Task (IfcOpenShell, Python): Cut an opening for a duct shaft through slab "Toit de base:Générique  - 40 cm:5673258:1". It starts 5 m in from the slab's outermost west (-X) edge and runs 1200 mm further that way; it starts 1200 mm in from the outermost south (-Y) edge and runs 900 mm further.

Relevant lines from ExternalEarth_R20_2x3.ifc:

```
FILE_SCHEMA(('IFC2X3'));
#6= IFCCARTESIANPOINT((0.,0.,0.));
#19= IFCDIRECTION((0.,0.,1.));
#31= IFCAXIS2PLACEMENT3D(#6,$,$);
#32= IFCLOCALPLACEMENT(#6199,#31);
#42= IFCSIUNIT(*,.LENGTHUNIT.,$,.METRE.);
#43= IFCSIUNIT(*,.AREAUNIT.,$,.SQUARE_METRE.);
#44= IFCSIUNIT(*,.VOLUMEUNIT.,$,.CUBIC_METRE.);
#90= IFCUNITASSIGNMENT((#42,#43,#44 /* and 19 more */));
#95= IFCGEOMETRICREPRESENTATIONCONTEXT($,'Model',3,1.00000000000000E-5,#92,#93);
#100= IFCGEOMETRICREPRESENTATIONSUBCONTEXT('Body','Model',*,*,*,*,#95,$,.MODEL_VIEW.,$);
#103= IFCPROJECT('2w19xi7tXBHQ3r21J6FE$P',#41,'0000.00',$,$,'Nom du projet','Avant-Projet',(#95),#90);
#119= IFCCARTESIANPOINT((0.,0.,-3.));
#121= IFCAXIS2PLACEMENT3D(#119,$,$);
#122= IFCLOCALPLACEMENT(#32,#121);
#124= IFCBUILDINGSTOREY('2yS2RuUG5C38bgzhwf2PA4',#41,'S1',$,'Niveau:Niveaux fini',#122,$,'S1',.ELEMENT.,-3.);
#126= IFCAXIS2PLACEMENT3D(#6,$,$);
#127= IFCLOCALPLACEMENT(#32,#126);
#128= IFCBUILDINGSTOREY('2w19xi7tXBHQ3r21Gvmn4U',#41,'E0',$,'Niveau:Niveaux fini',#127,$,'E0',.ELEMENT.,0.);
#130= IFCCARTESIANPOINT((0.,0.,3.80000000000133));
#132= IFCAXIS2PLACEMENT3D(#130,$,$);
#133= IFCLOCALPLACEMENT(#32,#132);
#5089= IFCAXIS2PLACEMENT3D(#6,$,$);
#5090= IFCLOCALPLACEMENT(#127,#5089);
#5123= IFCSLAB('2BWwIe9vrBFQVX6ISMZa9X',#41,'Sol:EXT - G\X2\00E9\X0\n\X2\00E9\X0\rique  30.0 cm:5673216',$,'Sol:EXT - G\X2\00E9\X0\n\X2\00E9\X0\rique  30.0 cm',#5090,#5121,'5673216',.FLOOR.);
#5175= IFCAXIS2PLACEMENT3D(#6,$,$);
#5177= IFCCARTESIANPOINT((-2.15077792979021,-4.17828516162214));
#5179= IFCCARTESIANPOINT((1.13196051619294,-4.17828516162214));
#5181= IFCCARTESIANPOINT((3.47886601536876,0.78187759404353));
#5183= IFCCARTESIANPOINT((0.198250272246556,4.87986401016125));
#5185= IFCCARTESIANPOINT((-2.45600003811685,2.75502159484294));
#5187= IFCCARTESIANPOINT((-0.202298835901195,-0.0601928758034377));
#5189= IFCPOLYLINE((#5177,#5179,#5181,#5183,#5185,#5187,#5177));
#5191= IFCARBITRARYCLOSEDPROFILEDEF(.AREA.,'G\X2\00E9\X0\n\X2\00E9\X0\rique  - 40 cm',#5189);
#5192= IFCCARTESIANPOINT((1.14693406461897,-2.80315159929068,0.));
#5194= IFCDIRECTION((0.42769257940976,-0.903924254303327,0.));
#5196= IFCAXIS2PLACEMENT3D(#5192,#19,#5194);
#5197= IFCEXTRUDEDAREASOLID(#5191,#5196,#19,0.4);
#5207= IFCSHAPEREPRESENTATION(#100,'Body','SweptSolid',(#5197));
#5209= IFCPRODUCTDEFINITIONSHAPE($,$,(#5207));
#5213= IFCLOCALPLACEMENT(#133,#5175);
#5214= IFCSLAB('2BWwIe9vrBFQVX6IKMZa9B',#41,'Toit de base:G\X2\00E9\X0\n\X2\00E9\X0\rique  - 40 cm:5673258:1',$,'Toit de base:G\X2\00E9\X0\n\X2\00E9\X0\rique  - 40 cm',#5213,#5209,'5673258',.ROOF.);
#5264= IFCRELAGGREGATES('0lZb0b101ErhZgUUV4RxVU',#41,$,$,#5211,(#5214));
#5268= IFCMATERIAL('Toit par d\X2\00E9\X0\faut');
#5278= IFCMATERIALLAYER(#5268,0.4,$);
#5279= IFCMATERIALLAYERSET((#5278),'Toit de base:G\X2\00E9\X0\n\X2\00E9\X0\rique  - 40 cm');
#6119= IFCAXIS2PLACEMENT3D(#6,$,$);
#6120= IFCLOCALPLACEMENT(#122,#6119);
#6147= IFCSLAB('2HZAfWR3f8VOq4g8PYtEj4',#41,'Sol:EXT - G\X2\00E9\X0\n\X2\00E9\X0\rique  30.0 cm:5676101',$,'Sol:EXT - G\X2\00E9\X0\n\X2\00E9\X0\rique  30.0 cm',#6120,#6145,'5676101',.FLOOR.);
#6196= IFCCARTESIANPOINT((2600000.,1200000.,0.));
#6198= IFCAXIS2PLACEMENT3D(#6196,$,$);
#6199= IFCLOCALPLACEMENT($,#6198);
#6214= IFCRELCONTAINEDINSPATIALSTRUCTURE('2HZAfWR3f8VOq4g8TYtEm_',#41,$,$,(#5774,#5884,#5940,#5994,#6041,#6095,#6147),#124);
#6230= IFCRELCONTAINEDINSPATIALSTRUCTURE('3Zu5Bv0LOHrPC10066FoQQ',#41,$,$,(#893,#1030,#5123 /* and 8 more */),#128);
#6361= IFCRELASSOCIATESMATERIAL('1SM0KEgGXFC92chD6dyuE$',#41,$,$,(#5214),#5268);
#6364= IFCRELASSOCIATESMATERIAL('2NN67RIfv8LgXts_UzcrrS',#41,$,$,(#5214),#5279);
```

```python
import numpy as np
import ifcopenshell
import ifcopenshell.api.feature
import ifcopenshell.api.geometry
import ifcopenshell.api.root
import ifcopenshell.geom
import ifcopenshell.util.placement
import ifcopenshell.util.representation
import ifcopenshell.util.shape
import ifcopenshell.util.unit

model = ifcopenshell.open("ExternalEarth_R20_2x3.ifc")
unit_scale = ifcopenshell.util.unit.calculate_unit_scale(model)
settings = ifcopenshell.geom.settings()


def volume(element):
    """Net volume in cubic metres, openings subtracted."""
    shape = ifcopenshell.geom.create_shape(settings, element)
    return ifcopenshell.util.shape.get_volume(shape.geometry)


slab = model.by_guid("2BWwIe9vrBFQVX6IKMZa9B")
before = volume(slab)

# Extent in the slab's own axes, in metres. The edges named are its -X and -Y sides.
slab_shape = ifcopenshell.geom.create_shape(settings, slab)
vertices = ifcopenshell.util.shape.get_vertices(slab_shape.geometry)
x_min, y_min, bottom = vertices.min(axis=0)
top = vertices[:, 2].max()

opening = ifcopenshell.api.root.create_entity(model, ifc_class="IfcOpeningElement", name="Duct shaft opening")
context = ifcopenshell.util.representation.get_context(model, "Model", "Body", "MODEL_VIEW")
width, depth = 1.2, 0.9
outline = [(0.0, 0.0), (width, 0.0), (width, depth), (0.0, depth), (0.0, 0.0)]
# Overshoot both faces by 50 mm so the cut is clean.
shape = ifcopenshell.api.geometry.add_slab_representation(
    model, context=context, depth=top - bottom + 0.1, polyline=outline
)
ifcopenshell.api.geometry.assign_representation(model, product=opening, representation=shape)

matrix = ifcopenshell.util.placement.get_local_placement(slab.ObjectPlacement)
matrix[:, 3] = matrix @ np.append(np.array([x_min + 5, y_min + 1.2, bottom - 0.05]) / unit_scale, 1.0)
ifcopenshell.api.geometry.edit_object_placement(model, product=opening, matrix=matrix, is_si=False)
ifcopenshell.api.feature.add_feature(model, feature=opening, element=slab)

after = volume(slab)

print(f"slab volume {before:.3f} -> {after:.3f} m3")

model.write("ExternalEarth_R20_2x3_updated.ifc")
```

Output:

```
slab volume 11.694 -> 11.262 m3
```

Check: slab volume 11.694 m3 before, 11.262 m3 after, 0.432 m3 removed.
